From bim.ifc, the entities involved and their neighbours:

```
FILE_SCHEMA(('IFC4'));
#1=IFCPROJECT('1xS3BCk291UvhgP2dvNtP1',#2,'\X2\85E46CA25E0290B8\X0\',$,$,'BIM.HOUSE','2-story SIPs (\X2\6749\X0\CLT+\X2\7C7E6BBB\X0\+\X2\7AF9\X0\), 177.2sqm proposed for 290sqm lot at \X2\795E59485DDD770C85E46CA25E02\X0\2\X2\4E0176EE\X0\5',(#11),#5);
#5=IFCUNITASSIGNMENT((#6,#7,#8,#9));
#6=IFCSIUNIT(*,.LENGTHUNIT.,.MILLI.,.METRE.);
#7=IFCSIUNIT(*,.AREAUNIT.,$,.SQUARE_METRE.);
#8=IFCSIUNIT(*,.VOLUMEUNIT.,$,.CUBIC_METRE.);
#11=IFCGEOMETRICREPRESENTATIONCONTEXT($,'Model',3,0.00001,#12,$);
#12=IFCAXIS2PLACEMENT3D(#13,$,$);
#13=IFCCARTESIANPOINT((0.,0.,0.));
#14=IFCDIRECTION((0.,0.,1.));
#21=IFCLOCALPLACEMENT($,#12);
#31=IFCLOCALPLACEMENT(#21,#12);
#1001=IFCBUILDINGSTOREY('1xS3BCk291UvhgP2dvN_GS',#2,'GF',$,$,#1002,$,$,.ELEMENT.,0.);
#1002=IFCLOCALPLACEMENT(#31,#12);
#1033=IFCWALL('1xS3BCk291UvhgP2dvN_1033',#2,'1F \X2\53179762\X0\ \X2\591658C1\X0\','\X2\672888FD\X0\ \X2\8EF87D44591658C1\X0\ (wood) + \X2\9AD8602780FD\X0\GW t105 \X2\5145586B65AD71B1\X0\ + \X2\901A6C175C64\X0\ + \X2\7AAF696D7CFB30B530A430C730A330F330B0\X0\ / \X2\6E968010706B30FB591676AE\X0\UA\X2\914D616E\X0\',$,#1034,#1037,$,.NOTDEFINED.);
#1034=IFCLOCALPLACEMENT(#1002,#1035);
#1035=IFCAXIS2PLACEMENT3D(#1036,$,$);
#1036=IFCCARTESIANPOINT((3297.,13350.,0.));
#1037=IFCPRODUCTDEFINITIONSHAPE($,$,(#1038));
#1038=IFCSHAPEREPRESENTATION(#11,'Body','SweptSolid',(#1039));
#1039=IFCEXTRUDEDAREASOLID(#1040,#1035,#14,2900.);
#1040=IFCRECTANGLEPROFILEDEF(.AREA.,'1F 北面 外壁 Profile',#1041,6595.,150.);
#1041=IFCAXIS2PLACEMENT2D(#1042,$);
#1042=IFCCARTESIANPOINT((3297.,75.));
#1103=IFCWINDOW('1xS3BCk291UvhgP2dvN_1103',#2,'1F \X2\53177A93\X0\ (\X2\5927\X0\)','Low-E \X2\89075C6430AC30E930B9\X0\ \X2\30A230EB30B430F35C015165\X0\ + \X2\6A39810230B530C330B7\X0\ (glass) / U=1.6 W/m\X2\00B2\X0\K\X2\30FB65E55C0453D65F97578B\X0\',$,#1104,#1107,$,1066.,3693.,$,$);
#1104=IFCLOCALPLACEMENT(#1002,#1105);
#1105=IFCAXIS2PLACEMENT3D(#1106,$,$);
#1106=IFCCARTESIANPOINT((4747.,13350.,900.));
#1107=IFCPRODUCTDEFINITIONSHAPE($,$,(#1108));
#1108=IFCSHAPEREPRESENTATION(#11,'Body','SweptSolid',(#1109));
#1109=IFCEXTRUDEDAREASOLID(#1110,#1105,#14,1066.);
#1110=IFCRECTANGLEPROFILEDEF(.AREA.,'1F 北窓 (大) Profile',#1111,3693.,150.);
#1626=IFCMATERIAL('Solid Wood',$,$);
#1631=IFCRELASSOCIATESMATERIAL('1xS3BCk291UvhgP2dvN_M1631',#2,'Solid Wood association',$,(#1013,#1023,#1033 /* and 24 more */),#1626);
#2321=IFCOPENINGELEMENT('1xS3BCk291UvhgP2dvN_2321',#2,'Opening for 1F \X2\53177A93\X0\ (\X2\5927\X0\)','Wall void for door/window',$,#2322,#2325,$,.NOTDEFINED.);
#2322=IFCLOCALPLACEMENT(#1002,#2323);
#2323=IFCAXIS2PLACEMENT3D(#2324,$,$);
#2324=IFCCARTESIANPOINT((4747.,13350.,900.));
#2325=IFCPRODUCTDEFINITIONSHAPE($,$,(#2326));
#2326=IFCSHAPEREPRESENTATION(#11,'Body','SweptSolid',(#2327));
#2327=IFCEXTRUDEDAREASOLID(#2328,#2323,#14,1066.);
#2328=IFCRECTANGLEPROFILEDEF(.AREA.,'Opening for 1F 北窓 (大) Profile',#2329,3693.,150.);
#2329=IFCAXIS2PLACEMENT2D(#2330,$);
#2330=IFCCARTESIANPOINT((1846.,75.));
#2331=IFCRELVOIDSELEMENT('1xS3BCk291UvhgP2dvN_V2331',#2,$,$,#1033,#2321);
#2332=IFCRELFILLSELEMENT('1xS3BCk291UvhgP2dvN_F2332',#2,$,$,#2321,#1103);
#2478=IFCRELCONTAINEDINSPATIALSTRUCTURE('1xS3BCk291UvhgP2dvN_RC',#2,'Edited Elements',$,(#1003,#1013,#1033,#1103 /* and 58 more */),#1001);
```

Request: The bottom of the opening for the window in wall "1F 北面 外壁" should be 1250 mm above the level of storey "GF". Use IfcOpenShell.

```python
import numpy as np
import ifcopenshell
import ifcopenshell.api.geometry
import ifcopenshell.geom
import ifcopenshell.util.element
import ifcopenshell.util.placement
import ifcopenshell.util.shape
import ifcopenshell.util.unit

model = ifcopenshell.open("bim.ifc")
unit_scale = ifcopenshell.util.unit.calculate_unit_scale(model)

window = model.by_guid("1xS3BCk291UvhgP2dvN_1103")
opening = window.FillsVoids[0].RelatingOpeningElement
storey = ifcopenshell.util.element.get_container(window, ifc_class="IfcBuildingStorey")
level = ifcopenshell.util.placement.get_local_placement(storey.ObjectPlacement)[2, 3]

# The opening's origin need not be at the sill, so measure its lowest point.
shape = ifcopenshell.geom.create_shape(ifcopenshell.geom.settings(), opening)
bottom = ifcopenshell.util.shape.get_shape_bottom_elevation(shape, shape.geometry) / unit_scale
dz = level + 1250.0 - bottom

shift = np.array([0.0, 0.0, dz])
# The window is not placed relative to its opening, so move both.
for product in (opening, window):
    matrix = ifcopenshell.util.placement.get_local_placement(product.ObjectPlacement)
    matrix[:3, 3] += shift
    ifcopenshell.api.geometry.edit_object_placement(model, product=product, matrix=matrix, is_si=False)

print(f"moved by {dz * unit_scale:+.3f} m")

model.write("bim-out.ifc")
```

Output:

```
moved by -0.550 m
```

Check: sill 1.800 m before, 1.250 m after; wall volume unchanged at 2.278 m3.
